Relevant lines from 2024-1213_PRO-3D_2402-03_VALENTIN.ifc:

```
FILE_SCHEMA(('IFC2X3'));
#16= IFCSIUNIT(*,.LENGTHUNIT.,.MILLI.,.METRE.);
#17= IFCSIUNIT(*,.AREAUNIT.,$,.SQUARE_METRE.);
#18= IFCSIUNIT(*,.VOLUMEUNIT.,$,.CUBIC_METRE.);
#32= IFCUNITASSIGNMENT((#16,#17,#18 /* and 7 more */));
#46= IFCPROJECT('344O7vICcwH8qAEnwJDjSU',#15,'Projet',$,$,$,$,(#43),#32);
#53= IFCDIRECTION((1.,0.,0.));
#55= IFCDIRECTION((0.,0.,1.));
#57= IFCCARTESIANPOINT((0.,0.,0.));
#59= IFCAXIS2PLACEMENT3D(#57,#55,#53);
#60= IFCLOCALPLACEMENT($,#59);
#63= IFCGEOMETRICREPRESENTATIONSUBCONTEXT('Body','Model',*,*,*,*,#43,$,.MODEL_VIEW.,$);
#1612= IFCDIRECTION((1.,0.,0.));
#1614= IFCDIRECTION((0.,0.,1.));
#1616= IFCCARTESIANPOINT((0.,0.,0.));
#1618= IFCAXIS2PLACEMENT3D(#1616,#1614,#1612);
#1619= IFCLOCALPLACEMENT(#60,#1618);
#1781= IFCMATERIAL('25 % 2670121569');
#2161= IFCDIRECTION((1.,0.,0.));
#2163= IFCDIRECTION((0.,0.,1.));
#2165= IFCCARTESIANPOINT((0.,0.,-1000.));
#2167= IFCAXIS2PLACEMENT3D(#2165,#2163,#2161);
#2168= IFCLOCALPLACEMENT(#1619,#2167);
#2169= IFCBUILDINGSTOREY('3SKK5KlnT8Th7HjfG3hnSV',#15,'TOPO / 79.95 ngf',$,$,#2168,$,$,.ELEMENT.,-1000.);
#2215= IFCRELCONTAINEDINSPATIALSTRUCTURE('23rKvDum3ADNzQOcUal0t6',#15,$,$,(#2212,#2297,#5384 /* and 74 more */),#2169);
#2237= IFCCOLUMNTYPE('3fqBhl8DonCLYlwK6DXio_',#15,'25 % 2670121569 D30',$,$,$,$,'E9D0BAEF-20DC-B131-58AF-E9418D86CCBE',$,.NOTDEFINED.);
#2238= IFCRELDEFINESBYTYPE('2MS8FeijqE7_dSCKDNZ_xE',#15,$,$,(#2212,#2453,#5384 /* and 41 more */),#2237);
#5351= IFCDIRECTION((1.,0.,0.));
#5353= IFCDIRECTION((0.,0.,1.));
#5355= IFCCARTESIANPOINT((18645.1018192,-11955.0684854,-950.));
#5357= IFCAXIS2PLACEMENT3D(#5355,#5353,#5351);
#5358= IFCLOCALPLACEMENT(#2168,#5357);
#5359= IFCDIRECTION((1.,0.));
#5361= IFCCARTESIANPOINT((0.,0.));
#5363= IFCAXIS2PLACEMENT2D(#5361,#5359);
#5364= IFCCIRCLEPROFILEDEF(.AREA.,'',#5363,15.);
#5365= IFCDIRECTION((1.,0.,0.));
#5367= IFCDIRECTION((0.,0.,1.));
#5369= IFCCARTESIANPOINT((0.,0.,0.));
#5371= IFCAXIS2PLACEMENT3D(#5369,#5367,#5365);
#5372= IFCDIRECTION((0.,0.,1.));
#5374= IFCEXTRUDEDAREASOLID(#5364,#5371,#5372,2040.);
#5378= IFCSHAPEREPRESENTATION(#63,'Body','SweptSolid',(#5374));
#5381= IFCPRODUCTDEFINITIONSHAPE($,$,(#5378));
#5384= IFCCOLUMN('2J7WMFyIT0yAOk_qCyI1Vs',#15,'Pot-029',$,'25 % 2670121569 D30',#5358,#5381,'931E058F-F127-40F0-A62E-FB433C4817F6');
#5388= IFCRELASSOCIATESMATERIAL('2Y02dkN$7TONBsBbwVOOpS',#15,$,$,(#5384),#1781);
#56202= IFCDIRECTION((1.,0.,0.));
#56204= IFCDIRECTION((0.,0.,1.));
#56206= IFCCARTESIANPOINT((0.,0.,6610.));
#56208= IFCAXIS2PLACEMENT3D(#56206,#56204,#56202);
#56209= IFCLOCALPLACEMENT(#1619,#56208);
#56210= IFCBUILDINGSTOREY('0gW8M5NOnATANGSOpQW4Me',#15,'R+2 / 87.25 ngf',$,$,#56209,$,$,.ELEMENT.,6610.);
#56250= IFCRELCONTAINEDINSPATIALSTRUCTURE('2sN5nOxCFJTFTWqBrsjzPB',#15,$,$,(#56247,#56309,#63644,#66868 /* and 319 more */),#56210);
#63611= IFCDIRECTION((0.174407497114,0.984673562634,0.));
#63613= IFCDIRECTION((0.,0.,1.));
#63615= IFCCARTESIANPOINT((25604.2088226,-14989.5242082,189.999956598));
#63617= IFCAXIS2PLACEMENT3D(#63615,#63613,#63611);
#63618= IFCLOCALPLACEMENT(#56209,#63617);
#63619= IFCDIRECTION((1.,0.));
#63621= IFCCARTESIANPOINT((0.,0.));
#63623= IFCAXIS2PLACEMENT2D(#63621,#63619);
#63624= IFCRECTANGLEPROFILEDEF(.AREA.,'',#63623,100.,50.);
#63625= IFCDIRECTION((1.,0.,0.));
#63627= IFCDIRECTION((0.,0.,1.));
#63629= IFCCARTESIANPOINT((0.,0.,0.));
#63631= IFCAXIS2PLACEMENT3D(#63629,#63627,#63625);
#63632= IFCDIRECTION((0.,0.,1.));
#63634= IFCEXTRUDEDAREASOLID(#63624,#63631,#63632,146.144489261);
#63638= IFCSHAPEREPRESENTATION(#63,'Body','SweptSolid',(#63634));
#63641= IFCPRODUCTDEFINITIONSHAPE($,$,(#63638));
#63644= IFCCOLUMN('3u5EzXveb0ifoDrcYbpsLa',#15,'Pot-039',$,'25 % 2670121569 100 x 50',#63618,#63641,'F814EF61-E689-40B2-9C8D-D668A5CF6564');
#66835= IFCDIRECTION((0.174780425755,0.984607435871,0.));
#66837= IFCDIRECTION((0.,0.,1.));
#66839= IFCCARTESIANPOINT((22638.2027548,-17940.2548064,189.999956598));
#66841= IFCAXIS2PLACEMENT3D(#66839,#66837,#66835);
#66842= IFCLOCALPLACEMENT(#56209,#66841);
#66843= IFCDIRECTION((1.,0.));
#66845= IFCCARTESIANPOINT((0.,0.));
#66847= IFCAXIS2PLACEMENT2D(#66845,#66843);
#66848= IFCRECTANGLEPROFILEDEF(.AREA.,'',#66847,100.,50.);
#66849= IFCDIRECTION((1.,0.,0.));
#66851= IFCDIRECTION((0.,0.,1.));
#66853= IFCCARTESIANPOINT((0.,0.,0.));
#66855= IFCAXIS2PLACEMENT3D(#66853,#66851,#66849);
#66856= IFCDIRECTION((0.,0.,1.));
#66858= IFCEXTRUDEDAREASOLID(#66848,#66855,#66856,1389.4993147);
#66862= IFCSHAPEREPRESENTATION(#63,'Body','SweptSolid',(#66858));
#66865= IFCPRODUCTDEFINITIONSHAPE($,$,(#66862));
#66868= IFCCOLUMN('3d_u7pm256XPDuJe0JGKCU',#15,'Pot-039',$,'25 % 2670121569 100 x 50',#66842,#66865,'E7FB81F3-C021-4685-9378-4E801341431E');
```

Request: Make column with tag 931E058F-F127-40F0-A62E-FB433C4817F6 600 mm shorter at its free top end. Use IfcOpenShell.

```python
import ifcopenshell
import ifcopenshell.util.representation
import ifcopenshell.util.unit

model = ifcopenshell.open("2024-1213_PRO-3D_2402-03_VALENTIN.ifc")
unit_scale = ifcopenshell.util.unit.calculate_unit_scale(model)

member = model.by_guid("2J7WMFyIT0yAOk_qCyI1Vs")
change = -0.6 / unit_scale

# The extrusion runs towards the end named, so only its depth changes.
body = ifcopenshell.util.representation.get_representation(member, "Model", "Body")
solid = body.Items[0]
old_length = solid.Depth
solid.Depth += change

print(f"length {old_length:g} -> {solid.Depth:g}")

model.write("2024-1213_PRO-3D_2402-03_VALENTIN_v2.ifc")
```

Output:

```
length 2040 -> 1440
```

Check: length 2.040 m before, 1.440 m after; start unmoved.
